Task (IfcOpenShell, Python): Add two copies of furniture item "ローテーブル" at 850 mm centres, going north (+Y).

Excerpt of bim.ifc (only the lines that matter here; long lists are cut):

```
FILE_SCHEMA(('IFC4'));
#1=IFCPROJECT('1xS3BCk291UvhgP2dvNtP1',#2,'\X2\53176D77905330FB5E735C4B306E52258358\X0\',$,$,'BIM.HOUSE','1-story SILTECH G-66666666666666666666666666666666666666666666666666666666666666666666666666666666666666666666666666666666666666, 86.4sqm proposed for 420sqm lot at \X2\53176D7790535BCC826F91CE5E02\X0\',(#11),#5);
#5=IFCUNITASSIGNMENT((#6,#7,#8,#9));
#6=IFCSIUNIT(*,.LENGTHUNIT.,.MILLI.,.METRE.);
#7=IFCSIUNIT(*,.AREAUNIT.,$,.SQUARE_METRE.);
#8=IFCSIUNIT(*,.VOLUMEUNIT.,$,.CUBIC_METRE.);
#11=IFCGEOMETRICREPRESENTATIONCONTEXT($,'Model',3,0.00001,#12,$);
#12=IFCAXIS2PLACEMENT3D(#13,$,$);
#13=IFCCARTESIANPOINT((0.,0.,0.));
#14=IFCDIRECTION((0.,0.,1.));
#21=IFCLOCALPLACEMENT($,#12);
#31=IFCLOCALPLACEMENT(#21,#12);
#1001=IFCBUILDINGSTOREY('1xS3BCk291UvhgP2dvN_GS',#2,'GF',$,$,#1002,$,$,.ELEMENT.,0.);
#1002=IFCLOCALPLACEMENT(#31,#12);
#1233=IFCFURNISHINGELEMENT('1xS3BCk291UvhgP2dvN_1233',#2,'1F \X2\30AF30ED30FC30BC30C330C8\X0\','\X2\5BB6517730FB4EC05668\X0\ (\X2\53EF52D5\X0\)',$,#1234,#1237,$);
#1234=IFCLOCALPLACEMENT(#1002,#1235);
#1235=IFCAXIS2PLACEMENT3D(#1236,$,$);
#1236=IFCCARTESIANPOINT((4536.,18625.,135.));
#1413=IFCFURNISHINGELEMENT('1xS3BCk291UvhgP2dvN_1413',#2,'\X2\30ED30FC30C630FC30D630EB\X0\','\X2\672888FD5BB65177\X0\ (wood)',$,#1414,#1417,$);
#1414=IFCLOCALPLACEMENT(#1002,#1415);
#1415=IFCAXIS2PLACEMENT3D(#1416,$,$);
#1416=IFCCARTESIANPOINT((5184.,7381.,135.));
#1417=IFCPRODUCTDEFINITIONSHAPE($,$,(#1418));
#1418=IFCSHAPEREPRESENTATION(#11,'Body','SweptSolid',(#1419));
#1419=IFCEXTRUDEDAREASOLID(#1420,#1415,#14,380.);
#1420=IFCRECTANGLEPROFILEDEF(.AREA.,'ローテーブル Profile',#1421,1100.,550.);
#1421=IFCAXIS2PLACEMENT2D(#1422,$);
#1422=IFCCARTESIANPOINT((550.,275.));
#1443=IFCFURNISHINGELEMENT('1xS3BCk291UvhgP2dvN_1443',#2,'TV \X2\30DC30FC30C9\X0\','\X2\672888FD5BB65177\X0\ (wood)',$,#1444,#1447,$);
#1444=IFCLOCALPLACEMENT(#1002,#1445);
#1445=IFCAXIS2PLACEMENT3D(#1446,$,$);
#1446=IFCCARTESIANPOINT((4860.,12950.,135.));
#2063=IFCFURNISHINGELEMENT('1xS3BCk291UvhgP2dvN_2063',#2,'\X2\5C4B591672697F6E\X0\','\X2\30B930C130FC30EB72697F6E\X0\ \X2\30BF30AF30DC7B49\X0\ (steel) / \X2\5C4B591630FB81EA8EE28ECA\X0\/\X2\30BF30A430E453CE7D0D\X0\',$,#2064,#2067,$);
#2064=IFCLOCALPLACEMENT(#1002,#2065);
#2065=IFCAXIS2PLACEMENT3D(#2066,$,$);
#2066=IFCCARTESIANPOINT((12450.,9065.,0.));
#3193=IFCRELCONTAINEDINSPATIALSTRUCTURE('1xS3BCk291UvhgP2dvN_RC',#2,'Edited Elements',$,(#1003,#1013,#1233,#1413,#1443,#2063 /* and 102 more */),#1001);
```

```python
import numpy as np
import ifcopenshell
import ifcopenshell.api.geometry
import ifcopenshell.api.root
import ifcopenshell.util.element
import ifcopenshell.util.placement
import ifcopenshell.util.unit

model = ifcopenshell.open("bim.ifc")
unit_scale = ifcopenshell.util.unit.calculate_unit_scale(model)


def reuse_history(source, copy):
    """copy_class also copies each property set's owner history, people and application; keep the originals."""
    for rel in copy.IsDefinedBy:
        if rel.is_a("IfcRelDefinesByProperties") and (history := rel.RelatingPropertyDefinition.OwnerHistory):
            rel.RelatingPropertyDefinition.OwnerHistory = source.OwnerHistory
            ifcopenshell.util.element.remove_deep2(model, history)


source = model.by_guid("1xS3BCk291UvhgP2dvN_1413")
base = ifcopenshell.util.placement.get_local_placement(source.ObjectPlacement)
step = np.array([0.0, 1.0, 0.0]) * 0.85 / unit_scale

for i in range(1, 3):
    copy = ifcopenshell.api.root.copy_class(model, product=source)
    copy.Representation = ifcopenshell.util.element.copy_deep(
        model, source.Representation, exclude=["IfcGeometricRepresentationContext", "IfcRepresentationMap"]
    )
    reuse_history(source, copy)
    matrix = base.copy()
    matrix[:3, 3] += i * step
    print("added at", matrix[:3, 3].round(3) + 0.0)
    ifcopenshell.api.geometry.edit_object_placement(model, product=copy, matrix=matrix, is_si=False)

model.write("bim_updated.ifc")
```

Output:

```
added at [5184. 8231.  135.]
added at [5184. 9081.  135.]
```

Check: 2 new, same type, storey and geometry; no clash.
